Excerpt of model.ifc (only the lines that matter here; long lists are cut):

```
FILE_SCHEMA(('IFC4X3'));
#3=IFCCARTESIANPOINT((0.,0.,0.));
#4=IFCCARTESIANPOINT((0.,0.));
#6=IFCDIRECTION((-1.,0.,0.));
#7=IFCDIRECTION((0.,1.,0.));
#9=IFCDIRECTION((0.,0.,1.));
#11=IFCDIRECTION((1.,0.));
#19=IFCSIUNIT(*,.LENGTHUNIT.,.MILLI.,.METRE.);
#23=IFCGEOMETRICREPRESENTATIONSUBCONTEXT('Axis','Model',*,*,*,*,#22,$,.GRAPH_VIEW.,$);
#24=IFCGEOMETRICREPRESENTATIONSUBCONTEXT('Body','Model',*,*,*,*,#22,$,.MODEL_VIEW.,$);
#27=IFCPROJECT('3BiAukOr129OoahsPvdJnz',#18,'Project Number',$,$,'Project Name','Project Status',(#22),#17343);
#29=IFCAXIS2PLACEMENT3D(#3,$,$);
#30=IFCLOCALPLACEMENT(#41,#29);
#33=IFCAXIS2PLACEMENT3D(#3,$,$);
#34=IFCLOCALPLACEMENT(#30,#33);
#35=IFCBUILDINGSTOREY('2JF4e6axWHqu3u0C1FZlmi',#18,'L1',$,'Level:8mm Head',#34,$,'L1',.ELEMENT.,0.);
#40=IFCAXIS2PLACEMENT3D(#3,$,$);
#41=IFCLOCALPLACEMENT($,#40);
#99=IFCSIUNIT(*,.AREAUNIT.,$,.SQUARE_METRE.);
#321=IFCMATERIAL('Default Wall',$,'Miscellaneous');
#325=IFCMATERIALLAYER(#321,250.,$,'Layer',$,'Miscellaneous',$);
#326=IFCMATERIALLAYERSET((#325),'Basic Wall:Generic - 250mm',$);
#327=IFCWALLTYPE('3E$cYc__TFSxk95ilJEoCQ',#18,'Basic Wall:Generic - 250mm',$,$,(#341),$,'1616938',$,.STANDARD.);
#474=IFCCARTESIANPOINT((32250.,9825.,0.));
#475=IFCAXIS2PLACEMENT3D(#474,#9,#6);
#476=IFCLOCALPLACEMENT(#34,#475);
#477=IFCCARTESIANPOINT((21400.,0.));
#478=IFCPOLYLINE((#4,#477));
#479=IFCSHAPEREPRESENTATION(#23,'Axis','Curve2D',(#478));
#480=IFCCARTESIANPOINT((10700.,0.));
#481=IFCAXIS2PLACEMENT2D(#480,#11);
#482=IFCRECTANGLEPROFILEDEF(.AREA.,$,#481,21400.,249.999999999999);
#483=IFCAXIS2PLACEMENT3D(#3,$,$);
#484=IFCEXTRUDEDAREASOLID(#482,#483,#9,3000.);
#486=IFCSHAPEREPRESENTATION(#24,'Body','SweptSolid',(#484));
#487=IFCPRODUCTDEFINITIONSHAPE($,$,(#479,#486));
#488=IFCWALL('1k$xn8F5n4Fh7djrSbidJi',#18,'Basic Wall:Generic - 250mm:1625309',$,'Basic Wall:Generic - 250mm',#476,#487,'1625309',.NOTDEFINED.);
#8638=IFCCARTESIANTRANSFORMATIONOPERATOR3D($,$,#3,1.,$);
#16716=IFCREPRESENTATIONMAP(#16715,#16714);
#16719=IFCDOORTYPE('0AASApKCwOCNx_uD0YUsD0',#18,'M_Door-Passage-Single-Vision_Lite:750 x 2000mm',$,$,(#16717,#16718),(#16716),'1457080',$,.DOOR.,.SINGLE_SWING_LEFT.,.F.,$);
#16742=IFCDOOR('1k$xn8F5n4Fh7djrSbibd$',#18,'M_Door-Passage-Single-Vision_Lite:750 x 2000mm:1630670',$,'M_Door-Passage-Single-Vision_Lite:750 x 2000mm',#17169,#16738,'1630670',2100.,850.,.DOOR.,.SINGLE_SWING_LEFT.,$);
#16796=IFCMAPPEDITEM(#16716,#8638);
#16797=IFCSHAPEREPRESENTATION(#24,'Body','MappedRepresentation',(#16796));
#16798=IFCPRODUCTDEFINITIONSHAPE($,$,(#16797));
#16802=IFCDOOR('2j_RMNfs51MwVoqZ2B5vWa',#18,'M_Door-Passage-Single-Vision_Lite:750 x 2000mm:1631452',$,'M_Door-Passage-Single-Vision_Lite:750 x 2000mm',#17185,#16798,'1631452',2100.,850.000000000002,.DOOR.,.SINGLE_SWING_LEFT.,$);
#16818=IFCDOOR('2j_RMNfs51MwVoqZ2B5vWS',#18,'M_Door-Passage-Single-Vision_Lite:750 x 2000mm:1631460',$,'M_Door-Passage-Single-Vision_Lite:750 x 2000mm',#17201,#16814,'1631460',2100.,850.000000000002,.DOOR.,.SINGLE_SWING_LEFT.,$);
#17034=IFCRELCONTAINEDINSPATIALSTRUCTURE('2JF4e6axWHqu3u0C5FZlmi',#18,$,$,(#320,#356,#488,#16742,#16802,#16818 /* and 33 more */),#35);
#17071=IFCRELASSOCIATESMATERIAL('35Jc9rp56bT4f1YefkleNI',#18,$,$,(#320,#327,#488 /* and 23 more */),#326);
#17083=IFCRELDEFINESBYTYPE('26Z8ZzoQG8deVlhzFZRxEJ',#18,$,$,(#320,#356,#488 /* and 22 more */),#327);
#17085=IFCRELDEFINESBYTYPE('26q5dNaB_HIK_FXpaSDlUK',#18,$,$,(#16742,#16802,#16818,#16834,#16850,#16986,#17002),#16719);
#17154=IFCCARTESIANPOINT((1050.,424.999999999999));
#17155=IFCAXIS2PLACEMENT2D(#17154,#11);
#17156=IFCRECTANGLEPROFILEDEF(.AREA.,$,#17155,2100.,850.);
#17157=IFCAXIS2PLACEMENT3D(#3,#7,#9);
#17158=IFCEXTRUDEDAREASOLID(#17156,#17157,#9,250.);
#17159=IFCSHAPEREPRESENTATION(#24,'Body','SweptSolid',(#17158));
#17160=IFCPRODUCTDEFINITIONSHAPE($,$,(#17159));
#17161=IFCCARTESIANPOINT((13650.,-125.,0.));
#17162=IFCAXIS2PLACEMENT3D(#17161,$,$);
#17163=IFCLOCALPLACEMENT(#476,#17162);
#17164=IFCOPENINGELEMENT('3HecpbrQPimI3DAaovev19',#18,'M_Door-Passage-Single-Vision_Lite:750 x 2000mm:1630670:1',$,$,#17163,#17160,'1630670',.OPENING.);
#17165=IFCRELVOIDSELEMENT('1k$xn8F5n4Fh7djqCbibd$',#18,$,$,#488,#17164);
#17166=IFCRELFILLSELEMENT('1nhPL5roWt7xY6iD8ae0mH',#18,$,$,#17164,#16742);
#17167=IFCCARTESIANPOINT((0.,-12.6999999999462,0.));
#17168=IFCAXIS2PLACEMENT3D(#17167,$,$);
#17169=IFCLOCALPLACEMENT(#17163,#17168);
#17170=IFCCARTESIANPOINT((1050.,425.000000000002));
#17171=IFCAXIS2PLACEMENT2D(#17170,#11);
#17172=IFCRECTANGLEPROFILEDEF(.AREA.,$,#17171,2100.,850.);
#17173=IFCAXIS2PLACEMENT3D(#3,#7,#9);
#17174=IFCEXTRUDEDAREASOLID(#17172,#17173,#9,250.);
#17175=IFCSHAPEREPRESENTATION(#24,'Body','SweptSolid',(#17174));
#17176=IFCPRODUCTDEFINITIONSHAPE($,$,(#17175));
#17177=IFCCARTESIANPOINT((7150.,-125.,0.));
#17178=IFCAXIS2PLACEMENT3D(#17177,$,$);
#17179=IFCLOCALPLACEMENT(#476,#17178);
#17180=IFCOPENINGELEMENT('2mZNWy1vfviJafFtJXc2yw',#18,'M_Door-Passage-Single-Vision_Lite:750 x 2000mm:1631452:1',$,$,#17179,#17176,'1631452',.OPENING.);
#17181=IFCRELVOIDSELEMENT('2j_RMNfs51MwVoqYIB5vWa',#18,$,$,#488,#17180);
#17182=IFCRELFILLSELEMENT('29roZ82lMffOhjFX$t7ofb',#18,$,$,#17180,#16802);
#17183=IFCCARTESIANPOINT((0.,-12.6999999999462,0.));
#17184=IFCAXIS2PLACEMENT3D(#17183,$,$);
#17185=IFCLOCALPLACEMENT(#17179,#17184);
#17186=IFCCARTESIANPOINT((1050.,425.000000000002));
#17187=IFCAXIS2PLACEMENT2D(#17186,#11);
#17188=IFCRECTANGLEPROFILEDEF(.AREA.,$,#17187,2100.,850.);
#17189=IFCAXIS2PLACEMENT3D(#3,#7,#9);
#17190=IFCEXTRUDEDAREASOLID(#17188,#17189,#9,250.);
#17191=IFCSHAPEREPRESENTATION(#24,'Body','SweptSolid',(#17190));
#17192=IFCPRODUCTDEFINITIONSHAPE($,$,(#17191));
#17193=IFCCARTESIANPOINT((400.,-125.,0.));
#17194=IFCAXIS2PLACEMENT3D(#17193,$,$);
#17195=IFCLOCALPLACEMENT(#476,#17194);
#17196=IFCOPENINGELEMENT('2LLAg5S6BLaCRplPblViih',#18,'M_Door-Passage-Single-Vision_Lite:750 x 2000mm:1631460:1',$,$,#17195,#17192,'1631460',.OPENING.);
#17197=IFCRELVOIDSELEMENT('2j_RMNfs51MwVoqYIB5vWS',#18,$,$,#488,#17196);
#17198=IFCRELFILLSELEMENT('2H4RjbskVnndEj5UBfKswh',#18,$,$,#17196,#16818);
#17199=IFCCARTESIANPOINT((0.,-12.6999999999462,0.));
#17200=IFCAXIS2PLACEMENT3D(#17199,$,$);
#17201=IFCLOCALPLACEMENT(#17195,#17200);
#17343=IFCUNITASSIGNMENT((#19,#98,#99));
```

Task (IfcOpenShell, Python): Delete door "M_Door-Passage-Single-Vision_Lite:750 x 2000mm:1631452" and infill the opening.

```python
import ifcopenshell
import ifcopenshell.api.feature
import ifcopenshell.api.root
import ifcopenshell.geom
import ifcopenshell.util.shape

model = ifcopenshell.open("model.ifc")
settings = ifcopenshell.geom.settings()


def volume(element):
    """Net volume in cubic metres, openings subtracted."""
    shape = ifcopenshell.geom.create_shape(settings, element)
    return ifcopenshell.util.shape.get_volume(shape.geometry)


door = model.by_guid("2j_RMNfs51MwVoqZ2B5vWa")
opening = door.FillsVoids[0].RelatingOpeningElement
wall = opening.VoidsElements[0].RelatingBuildingElement
before = volume(wall)

ifcopenshell.api.root.remove_product(model, product=door)
ifcopenshell.api.feature.remove_feature(model, feature=opening)

after = volume(wall)

print(f"wall volume {before:.3f} -> {after:.3f} m3")

model.write("model_rev.ifc")
```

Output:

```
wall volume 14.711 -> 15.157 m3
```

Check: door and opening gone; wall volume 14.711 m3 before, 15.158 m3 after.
